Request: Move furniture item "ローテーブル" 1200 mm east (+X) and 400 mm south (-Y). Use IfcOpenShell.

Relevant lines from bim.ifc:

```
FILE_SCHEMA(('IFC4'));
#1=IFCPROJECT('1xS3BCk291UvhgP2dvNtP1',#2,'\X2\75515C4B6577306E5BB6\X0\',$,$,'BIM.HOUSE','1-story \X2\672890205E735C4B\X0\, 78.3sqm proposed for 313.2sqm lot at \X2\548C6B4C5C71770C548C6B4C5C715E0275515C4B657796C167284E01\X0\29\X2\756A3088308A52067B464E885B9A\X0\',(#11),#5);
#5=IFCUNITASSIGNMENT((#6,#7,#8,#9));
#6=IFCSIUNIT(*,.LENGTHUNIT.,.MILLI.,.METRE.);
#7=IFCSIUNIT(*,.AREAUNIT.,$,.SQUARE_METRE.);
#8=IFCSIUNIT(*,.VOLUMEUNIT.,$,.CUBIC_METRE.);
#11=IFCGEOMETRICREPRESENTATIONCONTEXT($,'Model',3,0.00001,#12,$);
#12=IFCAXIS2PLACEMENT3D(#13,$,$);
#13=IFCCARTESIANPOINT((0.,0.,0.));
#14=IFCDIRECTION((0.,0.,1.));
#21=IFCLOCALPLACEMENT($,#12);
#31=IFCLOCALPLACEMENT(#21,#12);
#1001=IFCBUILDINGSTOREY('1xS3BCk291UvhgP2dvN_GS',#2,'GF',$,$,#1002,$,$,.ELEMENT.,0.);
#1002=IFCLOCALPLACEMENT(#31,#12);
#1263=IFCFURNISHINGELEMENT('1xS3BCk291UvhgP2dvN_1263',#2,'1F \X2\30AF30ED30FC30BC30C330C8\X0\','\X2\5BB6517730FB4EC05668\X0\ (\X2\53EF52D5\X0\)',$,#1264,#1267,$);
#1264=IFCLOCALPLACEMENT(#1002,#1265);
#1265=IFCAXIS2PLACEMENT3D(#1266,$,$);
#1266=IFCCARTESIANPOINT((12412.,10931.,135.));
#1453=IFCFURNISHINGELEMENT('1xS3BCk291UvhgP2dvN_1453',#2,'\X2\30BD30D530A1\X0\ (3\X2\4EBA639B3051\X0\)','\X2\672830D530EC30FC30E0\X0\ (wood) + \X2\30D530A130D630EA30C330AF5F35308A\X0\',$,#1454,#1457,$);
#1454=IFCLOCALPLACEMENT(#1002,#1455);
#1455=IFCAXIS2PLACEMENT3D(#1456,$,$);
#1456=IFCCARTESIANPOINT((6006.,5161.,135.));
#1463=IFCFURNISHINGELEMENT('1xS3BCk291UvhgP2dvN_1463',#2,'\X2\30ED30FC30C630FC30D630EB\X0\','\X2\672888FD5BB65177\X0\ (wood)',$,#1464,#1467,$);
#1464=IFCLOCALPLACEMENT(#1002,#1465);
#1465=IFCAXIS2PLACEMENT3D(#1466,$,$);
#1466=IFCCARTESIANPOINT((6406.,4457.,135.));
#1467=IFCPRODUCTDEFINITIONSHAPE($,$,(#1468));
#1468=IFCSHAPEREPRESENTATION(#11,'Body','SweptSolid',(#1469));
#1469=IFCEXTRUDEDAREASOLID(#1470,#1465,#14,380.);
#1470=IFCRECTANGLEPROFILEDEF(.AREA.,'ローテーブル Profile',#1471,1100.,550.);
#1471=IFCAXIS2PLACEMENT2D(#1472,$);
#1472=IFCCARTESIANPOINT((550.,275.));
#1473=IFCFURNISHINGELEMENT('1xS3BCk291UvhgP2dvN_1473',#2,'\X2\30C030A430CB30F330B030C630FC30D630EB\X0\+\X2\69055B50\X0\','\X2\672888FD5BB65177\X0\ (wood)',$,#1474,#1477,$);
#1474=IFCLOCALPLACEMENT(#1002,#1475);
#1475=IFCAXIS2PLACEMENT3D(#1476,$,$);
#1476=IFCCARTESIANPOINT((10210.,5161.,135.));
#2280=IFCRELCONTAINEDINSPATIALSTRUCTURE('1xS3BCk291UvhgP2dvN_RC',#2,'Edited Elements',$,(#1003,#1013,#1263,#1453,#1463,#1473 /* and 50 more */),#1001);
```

```python
import ifcopenshell
import ifcopenshell.api.geometry
import ifcopenshell.util.placement
import ifcopenshell.util.unit

model = ifcopenshell.open("bim.ifc")
unit_scale = ifcopenshell.util.unit.calculate_unit_scale(model)

item = model.by_id(1463)
matrix = ifcopenshell.util.placement.get_local_placement(item.ObjectPlacement)
matrix[0, 3] += 1.2 / unit_scale
matrix[1, 3] -= 0.4 / unit_scale
ifcopenshell.api.geometry.edit_object_placement(model, product=item, matrix=matrix, is_si=False)

print(ifcopenshell.util.placement.get_local_placement(item.ObjectPlacement).round(3) + 0.0)

model.write("bim_rev.ifc")
```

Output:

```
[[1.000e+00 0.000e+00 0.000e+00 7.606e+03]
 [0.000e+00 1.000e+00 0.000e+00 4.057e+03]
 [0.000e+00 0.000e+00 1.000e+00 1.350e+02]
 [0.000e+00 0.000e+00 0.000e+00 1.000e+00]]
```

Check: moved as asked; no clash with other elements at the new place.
